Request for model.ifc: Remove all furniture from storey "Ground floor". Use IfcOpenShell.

First a look at what the model holds.

```python
import ifcopenshell
import ifcopenshell.util.element

model = ifcopenshell.open("model.ifc")
print(model.schema)
storey = next(s for s in model.by_type("IfcBuildingStorey") if s.Name == "Ground floor")
furniture = [e for e in ifcopenshell.util.element.get_decomposition(storey) if e.is_a("IfcFurnishingElement")]
seen = {}
for e in furniture:
    element_type = ifcopenshell.util.element.get_type(e)
    name = element_type.Name if element_type not in (None, e) else None
    seen[name] = seen.get(name, 0) + 1
for name, count in sorted(seen.items(), key=str):
    print(count, "x", name)
```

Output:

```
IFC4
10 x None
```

```python
import ifcopenshell
import ifcopenshell.api.root
import ifcopenshell.util.element

model = ifcopenshell.open("model.ifc")

storey = next(s for s in model.by_type("IfcBuildingStorey") if s.Name == "Ground floor")
furniture = [e for e in ifcopenshell.util.element.get_decomposition(storey) if e.is_a("IfcFurnishingElement")]

for e in furniture:
    ifcopenshell.api.root.remove_product(model, product=e)
print(len(furniture), "removed")

model.write("model_updated.ifc")
```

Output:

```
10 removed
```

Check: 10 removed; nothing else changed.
